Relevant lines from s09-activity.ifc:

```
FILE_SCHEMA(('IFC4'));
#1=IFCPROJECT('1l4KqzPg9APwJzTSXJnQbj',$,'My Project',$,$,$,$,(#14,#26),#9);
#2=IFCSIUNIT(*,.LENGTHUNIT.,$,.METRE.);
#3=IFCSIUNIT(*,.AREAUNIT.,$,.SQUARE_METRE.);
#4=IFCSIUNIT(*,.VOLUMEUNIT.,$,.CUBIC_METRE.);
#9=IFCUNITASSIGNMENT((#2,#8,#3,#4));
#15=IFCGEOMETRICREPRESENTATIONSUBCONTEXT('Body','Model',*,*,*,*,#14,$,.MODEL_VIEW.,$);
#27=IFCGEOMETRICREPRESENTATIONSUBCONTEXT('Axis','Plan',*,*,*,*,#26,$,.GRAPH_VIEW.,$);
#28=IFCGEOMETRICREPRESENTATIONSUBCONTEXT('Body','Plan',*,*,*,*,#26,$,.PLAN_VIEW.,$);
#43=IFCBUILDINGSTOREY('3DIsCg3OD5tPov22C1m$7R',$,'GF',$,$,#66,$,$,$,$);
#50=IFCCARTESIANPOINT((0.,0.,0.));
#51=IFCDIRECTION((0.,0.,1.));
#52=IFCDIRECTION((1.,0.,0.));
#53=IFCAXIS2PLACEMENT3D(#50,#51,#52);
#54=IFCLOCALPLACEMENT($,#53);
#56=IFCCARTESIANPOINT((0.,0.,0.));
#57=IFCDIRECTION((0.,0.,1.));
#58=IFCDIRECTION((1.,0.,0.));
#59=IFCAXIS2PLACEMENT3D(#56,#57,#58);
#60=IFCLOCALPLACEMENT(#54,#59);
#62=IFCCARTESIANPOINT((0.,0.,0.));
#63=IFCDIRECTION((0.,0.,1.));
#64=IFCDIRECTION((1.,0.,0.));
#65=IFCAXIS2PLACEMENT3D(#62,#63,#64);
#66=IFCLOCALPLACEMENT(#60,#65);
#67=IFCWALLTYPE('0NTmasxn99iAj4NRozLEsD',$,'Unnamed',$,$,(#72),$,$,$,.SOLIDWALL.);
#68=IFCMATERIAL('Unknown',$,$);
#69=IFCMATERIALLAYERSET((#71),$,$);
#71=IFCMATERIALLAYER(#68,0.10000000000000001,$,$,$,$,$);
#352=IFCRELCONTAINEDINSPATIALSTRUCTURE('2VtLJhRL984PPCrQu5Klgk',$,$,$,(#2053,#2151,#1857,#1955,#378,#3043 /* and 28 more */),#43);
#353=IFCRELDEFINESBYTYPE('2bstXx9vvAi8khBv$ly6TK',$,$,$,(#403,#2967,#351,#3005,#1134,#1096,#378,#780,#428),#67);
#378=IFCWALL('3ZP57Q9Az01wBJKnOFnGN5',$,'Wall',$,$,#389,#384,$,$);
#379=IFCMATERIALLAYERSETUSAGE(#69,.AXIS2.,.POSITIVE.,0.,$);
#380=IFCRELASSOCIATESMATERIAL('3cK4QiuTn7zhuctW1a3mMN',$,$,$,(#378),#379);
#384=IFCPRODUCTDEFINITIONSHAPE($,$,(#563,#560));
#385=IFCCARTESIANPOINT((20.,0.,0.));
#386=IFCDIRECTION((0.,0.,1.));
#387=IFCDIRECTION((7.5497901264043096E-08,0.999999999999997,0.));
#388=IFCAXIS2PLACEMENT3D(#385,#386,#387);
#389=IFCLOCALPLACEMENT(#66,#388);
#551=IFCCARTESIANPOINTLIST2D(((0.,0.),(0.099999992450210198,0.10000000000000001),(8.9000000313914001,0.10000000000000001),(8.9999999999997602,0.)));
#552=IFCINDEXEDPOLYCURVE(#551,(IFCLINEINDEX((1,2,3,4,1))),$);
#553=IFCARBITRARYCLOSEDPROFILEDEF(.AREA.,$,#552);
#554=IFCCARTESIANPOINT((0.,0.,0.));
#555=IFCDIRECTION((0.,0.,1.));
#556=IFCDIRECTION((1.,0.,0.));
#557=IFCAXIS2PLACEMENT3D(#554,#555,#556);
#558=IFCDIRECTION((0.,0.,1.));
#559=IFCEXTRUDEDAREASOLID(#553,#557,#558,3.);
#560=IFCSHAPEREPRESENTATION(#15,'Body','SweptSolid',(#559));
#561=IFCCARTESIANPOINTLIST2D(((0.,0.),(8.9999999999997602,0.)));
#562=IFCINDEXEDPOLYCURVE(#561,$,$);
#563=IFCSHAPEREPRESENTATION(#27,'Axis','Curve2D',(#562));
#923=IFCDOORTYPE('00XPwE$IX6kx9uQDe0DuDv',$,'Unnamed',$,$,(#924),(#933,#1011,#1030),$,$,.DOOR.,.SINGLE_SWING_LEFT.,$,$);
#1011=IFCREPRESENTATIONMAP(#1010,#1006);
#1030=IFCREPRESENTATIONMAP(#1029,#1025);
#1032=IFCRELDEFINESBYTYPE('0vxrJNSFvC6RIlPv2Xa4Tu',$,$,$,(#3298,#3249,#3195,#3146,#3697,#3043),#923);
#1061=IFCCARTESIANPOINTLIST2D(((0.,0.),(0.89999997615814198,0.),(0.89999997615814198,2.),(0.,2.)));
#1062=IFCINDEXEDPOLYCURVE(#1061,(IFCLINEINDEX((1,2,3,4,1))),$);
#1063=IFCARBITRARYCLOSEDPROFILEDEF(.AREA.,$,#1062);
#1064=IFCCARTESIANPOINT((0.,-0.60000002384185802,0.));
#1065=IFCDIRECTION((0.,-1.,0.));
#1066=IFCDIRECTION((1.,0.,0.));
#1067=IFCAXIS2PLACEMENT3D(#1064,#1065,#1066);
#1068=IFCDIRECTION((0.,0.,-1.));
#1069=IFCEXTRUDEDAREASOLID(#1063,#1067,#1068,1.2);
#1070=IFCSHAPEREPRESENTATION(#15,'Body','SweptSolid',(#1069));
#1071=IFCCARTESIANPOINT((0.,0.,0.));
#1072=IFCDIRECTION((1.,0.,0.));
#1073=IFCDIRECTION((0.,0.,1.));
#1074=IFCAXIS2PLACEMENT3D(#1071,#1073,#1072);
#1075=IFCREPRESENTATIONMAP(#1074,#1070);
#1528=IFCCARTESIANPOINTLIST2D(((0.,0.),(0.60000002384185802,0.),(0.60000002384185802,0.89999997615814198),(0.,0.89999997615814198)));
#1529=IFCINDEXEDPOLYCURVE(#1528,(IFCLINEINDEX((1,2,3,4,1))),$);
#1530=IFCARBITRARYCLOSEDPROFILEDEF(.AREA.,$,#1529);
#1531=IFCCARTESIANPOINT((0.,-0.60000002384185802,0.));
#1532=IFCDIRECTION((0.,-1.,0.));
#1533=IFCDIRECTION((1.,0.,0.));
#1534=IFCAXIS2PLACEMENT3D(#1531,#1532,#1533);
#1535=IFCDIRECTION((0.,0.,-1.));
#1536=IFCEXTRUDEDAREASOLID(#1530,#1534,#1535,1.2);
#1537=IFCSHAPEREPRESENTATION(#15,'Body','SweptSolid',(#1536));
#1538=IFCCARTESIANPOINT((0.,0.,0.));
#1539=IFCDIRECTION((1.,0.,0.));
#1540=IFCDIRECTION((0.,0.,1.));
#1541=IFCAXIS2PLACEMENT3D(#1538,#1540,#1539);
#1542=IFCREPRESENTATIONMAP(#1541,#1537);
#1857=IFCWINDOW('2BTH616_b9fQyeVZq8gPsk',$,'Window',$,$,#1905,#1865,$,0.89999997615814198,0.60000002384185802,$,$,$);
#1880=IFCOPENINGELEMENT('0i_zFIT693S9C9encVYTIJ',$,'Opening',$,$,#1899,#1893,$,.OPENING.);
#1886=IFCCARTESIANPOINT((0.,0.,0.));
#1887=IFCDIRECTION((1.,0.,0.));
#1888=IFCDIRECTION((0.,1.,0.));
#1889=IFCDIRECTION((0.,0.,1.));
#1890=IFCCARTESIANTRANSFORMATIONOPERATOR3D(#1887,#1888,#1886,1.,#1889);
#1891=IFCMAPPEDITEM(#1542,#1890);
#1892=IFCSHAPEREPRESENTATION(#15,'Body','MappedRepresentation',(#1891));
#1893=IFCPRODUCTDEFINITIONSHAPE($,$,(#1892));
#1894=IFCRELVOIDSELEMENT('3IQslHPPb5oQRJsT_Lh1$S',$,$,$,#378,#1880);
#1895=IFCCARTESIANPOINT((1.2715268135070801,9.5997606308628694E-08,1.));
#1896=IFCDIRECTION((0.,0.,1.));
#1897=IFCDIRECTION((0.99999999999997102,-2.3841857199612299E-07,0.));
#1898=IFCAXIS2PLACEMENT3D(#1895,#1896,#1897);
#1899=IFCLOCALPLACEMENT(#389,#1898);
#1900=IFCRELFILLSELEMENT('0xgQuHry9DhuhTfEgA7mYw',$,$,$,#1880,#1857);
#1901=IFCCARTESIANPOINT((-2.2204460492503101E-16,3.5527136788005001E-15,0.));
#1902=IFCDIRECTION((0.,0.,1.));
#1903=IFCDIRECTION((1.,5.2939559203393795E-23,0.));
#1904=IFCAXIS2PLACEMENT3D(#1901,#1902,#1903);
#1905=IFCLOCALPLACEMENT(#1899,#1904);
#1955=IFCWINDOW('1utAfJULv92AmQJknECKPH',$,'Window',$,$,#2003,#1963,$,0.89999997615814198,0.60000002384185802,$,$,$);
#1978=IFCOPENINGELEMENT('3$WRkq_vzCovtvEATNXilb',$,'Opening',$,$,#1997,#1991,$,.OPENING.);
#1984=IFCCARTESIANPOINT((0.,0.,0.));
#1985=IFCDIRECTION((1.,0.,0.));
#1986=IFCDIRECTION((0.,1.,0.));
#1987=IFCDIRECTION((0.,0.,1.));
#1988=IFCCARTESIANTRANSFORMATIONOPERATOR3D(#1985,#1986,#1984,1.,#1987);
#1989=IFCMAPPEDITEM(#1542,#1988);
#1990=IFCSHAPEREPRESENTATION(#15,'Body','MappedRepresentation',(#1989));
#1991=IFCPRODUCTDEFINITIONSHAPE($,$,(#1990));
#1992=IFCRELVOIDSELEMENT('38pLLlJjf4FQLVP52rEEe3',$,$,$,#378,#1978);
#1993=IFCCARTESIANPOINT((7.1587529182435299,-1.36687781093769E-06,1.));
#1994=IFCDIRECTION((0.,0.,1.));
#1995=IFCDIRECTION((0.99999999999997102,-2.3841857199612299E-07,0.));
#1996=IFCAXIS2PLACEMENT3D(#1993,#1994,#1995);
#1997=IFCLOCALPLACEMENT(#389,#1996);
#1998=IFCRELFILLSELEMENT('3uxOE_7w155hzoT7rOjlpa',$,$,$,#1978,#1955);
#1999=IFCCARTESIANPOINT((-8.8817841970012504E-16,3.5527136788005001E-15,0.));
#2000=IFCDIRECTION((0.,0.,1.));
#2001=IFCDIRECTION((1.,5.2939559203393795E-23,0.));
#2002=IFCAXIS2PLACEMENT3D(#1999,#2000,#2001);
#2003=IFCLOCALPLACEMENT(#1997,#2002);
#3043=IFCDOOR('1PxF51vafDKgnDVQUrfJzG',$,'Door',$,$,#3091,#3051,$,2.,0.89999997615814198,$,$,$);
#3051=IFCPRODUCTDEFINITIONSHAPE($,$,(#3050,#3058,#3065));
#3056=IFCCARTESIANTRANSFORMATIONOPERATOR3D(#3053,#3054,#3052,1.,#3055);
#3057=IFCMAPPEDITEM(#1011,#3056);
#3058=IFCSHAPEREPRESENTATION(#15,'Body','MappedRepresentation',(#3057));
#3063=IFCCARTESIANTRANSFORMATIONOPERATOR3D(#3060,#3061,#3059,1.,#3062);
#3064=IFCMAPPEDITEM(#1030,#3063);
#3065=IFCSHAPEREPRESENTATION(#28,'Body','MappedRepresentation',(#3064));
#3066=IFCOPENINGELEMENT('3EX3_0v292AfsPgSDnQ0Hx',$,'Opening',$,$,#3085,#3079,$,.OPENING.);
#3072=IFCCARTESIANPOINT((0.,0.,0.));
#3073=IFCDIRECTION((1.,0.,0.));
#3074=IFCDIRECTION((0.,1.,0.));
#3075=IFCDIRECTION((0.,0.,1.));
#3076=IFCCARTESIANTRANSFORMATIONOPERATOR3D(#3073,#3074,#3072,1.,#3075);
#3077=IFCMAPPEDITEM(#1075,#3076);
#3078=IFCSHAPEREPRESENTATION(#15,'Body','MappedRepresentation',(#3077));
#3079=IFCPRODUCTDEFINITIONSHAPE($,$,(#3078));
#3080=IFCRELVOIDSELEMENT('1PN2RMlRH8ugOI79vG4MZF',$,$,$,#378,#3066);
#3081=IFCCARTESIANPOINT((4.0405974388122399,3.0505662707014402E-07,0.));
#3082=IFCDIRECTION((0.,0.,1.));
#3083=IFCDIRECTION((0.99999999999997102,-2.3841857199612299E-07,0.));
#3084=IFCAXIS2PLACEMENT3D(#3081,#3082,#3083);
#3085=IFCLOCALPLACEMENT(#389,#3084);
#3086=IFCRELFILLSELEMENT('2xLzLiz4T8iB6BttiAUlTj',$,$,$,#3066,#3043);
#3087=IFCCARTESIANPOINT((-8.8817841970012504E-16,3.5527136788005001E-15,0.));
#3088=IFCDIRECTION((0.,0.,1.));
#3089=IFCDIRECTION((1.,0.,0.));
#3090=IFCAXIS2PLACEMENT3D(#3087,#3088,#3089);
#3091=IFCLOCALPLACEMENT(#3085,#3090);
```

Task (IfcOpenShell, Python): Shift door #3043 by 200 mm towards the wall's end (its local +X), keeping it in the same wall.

```python
import ifcopenshell
import ifcopenshell.api.geometry
import ifcopenshell.util.placement

model = ifcopenshell.open("s09-activity.ifc")

door = model.by_guid("1PxF51vafDKgnDVQUrfJzG")
opening = door.FillsVoids[0].RelatingOpeningElement
wall = opening.VoidsElements[0].RelatingBuildingElement

wall_matrix = ifcopenshell.util.placement.get_local_placement(wall.ObjectPlacement)
shift = wall_matrix[:3, 0] * 0.2
before = ifcopenshell.util.placement.get_local_placement(door.ObjectPlacement)[:3, 3].copy()

# The door is placed relative to its opening, so it follows when the opening moves.
matrix = ifcopenshell.util.placement.get_local_placement(opening.ObjectPlacement)
matrix[:3, 3] += shift
ifcopenshell.api.geometry.edit_object_placement(
    model, product=opening, matrix=matrix, is_si=False, should_transform_children=True
)

after = ifcopenshell.util.placement.get_local_placement(door.ObjectPlacement)[:3, 3]
print("door moved by", (after - before).round(3) + 0.0)

model.write("s09-activity_rev.ifc")
```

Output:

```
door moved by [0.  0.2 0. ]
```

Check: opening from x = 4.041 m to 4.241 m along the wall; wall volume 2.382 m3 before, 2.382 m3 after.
